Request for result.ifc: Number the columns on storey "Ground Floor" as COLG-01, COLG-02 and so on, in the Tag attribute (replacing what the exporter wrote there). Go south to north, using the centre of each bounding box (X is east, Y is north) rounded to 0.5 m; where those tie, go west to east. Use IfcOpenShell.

First a look at what the model holds.

```python
import ifcopenshell
import ifcopenshell.util.element
import ifcopenshell.util.placement

model = ifcopenshell.open("result.ifc")
print(model.schema)
storey = next(s for s in model.by_type("IfcBuildingStorey") if s.Name == "Ground Floor")
columns = [e for e in ifcopenshell.util.element.get_decomposition(storey) if e.is_a("IfcColumn")]
for e in sorted(columns, key=lambda e: e.id()):
    origin = ifcopenshell.util.placement.get_local_placement(e.ObjectPlacement)[:3, 3]
    print(e.id(), e.Tag, e.Name, origin.round(2) + 0.0, sep=" | ")
```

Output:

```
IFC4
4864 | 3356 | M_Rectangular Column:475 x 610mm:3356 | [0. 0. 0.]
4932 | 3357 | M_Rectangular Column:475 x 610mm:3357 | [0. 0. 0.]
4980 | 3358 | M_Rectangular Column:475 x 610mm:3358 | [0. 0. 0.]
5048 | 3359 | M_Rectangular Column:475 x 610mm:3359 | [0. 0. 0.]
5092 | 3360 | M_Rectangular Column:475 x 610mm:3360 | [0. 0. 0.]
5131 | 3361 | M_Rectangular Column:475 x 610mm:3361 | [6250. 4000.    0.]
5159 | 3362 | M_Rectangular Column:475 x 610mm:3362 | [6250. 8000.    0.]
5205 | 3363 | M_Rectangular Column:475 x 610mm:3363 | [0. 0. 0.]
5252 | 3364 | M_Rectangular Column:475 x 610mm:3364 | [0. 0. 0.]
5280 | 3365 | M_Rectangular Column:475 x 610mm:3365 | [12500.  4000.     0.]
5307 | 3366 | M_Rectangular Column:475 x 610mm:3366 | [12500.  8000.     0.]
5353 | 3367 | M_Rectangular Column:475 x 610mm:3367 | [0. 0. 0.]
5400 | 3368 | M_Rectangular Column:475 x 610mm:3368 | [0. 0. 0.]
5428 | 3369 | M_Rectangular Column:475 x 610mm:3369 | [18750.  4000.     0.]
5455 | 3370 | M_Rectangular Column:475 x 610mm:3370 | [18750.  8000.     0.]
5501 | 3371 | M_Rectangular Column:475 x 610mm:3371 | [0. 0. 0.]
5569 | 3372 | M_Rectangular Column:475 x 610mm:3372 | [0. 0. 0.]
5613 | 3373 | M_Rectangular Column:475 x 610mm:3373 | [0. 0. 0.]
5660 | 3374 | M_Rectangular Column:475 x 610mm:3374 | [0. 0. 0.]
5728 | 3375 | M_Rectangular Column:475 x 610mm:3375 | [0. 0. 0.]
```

```python
import ifcopenshell
import ifcopenshell.geom
import ifcopenshell.util.element
import ifcopenshell.util.shape

model = ifcopenshell.open("result.ifc")
settings = ifcopenshell.geom.settings()
settings.set("use-world-coords", True)


def centre(element):
    shape = ifcopenshell.geom.create_shape(settings, element)
    return ifcopenshell.util.shape.get_bbox_centroid(shape.geometry)


storey = next(s for s in model.by_type("IfcBuildingStorey") if s.Name == "Ground Floor")
columns = [e for e in ifcopenshell.util.element.get_decomposition(storey) if e.is_a("IfcColumn")]

# Insertion points can sit at a corner or the storey origin, so sort by the geometry (in metres).
centres = {e: centre(e) for e in columns}
columns.sort(key=lambda e: (round(centres[e][1] / 0.5), centres[e][0]))

for i, e in enumerate(columns, start=1):
    number = f"COLG-{i:02d}"
    e.Tag = number
    print(e.id(), number)

model.write("result_updated.ifc")
```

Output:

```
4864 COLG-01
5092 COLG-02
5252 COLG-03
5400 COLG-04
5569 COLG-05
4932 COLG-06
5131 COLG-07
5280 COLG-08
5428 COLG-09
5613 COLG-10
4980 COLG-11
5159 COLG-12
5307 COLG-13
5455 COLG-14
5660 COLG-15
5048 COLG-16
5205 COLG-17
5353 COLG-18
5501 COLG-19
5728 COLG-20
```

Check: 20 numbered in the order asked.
